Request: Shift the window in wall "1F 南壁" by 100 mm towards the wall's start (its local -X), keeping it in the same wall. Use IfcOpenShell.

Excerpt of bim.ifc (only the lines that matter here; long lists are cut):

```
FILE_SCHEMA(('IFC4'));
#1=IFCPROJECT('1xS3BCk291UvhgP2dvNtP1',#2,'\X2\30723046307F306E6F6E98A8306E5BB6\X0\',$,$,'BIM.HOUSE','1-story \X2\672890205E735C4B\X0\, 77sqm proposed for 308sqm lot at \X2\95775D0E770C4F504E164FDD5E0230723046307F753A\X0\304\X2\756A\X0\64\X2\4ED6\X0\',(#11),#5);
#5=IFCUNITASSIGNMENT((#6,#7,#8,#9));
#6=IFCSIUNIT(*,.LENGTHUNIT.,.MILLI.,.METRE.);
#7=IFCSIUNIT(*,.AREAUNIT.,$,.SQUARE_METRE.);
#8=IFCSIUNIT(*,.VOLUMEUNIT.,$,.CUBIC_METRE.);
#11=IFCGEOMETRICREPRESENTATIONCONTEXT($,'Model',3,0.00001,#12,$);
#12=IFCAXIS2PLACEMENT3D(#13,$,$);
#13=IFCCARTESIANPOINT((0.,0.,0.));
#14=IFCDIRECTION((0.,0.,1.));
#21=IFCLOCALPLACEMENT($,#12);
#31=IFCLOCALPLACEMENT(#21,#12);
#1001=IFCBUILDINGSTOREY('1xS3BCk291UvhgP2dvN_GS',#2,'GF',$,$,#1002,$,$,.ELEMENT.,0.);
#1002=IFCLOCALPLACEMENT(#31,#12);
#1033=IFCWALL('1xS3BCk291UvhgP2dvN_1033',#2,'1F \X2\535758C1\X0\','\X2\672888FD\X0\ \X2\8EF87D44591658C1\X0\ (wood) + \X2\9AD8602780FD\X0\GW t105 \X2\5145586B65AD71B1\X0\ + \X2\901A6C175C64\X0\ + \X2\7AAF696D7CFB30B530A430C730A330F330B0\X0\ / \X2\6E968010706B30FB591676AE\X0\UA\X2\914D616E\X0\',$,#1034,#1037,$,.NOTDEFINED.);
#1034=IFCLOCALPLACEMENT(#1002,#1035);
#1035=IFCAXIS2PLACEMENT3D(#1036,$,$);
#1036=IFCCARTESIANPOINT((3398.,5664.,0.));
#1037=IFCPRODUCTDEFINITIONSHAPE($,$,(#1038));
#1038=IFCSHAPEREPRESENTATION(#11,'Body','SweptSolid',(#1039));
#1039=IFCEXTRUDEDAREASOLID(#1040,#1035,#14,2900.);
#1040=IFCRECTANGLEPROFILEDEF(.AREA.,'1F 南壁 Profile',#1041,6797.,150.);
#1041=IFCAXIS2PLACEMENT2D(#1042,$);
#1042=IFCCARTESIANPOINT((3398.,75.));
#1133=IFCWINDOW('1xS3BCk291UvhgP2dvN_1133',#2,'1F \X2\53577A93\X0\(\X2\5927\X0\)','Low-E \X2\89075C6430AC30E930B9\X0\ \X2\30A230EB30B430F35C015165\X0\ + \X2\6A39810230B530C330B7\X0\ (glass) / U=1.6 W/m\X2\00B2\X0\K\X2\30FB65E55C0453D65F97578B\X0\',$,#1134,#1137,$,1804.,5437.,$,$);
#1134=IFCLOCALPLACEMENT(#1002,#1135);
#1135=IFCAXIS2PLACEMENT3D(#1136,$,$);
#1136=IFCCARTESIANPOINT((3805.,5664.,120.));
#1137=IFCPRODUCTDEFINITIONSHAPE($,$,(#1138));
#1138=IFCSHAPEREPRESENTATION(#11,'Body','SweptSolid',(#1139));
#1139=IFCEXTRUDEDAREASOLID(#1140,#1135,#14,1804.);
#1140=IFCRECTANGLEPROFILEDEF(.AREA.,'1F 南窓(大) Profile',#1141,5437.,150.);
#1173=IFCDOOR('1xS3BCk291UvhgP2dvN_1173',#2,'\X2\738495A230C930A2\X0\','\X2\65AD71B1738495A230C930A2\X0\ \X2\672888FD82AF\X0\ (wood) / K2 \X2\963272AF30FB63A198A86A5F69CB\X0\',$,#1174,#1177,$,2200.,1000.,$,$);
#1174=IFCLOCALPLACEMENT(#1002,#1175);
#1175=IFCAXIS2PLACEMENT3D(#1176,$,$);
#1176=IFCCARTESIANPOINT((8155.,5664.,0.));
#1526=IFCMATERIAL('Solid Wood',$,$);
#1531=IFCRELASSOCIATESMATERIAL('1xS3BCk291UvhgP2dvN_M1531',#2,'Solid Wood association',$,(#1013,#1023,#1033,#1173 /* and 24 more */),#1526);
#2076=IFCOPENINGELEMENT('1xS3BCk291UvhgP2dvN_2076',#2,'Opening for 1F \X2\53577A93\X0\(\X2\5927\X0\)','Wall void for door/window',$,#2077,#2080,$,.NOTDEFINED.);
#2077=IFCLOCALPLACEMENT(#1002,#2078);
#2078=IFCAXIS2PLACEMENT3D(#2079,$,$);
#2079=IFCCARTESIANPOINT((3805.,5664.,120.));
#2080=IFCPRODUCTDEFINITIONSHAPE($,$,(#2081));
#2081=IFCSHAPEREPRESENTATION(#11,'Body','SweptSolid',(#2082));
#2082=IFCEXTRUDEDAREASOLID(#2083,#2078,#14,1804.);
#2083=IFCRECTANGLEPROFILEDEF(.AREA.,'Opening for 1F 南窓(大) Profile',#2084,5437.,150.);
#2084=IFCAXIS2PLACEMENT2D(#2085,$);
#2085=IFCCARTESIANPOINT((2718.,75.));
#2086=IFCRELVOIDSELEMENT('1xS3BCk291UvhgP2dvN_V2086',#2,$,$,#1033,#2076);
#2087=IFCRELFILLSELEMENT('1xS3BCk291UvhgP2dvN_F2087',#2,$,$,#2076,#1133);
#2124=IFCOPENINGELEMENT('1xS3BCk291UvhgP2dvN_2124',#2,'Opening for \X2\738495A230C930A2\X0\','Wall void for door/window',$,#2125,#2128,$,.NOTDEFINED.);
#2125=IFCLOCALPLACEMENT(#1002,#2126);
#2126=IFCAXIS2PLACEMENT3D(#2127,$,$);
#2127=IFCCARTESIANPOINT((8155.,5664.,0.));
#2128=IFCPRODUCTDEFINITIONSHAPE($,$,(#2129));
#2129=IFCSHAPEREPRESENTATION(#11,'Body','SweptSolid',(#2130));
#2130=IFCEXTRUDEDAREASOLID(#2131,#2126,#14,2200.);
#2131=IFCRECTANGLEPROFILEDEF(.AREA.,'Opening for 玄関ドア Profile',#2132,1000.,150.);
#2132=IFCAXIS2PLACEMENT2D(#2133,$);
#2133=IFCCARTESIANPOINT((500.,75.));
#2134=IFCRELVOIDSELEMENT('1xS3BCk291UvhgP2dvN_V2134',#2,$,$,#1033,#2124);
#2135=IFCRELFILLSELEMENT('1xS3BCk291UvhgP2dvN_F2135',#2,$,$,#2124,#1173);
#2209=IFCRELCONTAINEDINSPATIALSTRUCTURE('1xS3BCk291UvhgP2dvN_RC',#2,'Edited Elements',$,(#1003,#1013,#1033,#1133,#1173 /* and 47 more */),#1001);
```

```python
import ifcopenshell
import ifcopenshell.api.geometry
import ifcopenshell.util.placement
import ifcopenshell.util.unit

model = ifcopenshell.open("bim.ifc")
unit_scale = ifcopenshell.util.unit.calculate_unit_scale(model)

window = model.by_guid("1xS3BCk291UvhgP2dvN_1133")
opening = window.FillsVoids[0].RelatingOpeningElement
wall = opening.VoidsElements[0].RelatingBuildingElement

wall_matrix = ifcopenshell.util.placement.get_local_placement(wall.ObjectPlacement)
shift = wall_matrix[:3, 0] * -0.1 / unit_scale
before = ifcopenshell.util.placement.get_local_placement(window.ObjectPlacement)[:3, 3].copy()

# The window is not placed relative to its opening, so move both.
for product in (opening, window):
    matrix = ifcopenshell.util.placement.get_local_placement(product.ObjectPlacement)
    matrix[:3, 3] += shift
    ifcopenshell.api.geometry.edit_object_placement(model, product=product, matrix=matrix, is_si=False)

after = ifcopenshell.util.placement.get_local_placement(window.ObjectPlacement)[:3, 3]
print("window moved by", (after - before).round(3) + 0.0)

model.write("bim_v2.ifc")
```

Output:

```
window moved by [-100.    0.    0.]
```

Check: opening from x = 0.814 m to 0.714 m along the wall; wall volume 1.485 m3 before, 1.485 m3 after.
